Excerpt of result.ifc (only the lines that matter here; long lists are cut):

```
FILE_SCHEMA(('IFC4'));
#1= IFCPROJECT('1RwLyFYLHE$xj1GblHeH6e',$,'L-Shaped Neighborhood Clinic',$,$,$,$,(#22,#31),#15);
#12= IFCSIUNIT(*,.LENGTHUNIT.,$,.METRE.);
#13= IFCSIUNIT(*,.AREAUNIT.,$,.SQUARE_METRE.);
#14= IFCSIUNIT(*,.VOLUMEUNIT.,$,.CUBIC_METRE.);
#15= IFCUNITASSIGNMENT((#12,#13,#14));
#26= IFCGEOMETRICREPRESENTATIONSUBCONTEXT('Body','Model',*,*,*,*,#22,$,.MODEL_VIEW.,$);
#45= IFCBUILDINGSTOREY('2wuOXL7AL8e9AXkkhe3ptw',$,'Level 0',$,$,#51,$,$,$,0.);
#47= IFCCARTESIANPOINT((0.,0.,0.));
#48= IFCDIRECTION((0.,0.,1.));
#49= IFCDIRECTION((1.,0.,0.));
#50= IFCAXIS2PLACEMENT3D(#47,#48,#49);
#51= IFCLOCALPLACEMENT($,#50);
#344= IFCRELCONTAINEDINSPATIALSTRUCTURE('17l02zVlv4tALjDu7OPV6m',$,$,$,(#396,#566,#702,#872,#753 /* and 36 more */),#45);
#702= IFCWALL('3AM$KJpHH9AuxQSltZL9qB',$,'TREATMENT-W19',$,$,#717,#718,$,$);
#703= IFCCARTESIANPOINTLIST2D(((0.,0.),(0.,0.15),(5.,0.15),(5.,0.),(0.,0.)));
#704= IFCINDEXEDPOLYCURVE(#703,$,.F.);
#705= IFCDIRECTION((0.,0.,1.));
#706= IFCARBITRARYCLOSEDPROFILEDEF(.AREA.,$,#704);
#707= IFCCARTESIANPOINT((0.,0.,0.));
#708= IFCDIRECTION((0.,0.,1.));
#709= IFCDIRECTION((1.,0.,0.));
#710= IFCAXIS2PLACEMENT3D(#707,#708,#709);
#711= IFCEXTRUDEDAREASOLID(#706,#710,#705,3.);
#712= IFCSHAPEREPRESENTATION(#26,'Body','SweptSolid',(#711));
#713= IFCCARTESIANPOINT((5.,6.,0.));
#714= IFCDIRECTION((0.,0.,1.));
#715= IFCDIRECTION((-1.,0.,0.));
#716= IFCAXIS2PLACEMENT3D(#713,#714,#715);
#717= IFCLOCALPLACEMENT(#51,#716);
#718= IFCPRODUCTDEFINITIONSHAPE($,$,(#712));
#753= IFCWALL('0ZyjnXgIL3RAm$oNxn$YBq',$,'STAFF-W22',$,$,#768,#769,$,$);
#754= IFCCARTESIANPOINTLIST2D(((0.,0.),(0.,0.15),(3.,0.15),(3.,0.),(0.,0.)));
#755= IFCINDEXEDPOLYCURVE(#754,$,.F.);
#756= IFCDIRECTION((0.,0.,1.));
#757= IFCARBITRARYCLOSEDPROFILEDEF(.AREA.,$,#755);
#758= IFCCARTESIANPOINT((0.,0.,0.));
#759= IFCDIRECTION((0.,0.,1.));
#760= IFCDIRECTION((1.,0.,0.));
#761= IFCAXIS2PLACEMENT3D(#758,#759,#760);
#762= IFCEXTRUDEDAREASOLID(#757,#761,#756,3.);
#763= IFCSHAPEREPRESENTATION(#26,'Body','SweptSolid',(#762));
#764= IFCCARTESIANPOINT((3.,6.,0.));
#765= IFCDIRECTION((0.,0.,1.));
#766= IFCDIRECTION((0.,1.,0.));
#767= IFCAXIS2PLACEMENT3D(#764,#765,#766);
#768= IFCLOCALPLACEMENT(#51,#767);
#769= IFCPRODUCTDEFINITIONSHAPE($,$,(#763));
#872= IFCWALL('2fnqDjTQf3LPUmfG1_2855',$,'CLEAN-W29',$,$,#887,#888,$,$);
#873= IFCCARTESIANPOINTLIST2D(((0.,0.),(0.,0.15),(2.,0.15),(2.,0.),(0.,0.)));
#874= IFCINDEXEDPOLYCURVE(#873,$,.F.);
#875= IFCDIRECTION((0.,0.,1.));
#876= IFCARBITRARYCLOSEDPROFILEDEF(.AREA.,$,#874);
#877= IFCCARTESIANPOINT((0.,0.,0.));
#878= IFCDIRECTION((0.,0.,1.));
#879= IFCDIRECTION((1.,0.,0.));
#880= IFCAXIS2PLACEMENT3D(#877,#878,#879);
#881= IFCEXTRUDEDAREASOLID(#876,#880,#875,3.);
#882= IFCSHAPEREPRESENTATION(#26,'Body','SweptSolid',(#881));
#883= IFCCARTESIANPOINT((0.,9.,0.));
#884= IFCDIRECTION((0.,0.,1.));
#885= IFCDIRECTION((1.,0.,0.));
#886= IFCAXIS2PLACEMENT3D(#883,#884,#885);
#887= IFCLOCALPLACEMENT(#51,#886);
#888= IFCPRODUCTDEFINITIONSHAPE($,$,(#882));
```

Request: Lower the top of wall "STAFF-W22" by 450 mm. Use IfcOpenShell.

```python
import ifcopenshell
import ifcopenshell.geom
import ifcopenshell.util.representation
import ifcopenshell.util.shape
import ifcopenshell.util.unit

model = ifcopenshell.open("result.ifc")
unit_scale = ifcopenshell.util.unit.calculate_unit_scale(model)
settings = ifcopenshell.geom.settings()


def volume(element):
    """Net volume in cubic metres, openings subtracted."""
    shape = ifcopenshell.geom.create_shape(settings, element)
    return ifcopenshell.util.shape.get_volume(shape.geometry)


wall = model.by_guid("0ZyjnXgIL3RAm$oNxn$YBq")
before = volume(wall)

body = ifcopenshell.util.representation.get_representation(wall, "Model", "Body")
solid = body.Items[0]
old_height = solid.Depth
solid.Depth -= 0.45 / unit_scale
after = volume(wall)

print(f"height {old_height:g} -> {solid.Depth:g}, volume {before:.3f} -> {after:.3f} m3")

model.write("result_rev.ifc")
```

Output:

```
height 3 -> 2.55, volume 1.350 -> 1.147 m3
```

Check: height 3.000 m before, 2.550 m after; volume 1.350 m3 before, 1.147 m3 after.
